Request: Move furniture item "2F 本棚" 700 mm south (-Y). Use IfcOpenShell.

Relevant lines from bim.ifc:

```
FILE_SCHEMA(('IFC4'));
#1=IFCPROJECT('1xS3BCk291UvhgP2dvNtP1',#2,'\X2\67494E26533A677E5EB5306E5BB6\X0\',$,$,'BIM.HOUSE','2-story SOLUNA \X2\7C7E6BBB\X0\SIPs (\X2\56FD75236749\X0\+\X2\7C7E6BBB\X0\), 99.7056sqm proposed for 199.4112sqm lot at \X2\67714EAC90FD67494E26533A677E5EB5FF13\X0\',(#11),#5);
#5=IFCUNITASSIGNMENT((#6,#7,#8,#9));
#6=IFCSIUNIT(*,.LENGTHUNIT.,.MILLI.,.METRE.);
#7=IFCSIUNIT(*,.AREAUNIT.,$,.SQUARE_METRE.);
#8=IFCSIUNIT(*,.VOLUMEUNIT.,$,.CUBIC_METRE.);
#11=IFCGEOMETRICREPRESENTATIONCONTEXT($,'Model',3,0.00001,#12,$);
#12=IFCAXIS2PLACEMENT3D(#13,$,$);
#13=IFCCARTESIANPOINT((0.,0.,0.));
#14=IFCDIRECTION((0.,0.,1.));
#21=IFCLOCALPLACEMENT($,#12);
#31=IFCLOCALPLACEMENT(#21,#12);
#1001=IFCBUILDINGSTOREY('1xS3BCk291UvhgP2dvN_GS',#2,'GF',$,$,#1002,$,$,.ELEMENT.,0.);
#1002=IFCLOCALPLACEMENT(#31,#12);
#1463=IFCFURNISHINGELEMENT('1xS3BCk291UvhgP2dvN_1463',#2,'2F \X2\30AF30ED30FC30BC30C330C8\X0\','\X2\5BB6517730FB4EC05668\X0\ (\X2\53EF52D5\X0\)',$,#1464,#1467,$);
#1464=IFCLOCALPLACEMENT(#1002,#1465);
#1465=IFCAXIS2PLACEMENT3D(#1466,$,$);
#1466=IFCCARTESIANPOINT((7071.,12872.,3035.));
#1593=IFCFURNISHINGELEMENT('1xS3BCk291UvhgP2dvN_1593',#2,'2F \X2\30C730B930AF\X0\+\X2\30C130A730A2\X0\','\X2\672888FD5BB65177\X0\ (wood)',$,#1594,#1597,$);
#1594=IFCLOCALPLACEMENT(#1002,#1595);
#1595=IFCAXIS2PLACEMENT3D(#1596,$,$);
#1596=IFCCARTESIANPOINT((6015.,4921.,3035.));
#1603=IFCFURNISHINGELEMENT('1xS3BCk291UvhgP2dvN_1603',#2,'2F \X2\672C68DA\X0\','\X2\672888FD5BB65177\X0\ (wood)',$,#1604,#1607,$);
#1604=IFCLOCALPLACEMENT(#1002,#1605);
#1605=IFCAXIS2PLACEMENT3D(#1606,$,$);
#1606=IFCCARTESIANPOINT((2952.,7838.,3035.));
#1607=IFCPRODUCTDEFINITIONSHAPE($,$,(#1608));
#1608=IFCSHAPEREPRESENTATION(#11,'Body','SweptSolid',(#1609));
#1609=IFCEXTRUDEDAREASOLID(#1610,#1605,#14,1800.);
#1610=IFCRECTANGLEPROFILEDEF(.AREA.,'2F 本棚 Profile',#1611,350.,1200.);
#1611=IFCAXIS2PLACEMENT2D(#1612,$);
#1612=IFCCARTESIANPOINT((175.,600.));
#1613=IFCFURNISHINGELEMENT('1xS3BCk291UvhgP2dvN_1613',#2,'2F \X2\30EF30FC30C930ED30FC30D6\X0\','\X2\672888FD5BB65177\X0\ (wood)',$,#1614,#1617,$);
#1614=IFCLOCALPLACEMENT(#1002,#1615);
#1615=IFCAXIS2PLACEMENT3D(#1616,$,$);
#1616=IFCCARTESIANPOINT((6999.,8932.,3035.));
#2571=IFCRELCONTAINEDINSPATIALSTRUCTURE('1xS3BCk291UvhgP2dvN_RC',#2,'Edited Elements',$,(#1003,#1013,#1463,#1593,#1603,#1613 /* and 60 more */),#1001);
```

```python
import ifcopenshell
import ifcopenshell.api.geometry
import ifcopenshell.util.placement
import ifcopenshell.util.unit

model = ifcopenshell.open("bim.ifc")
unit_scale = ifcopenshell.util.unit.calculate_unit_scale(model)

item = model.by_guid("1xS3BCk291UvhgP2dvN_1603")
matrix = ifcopenshell.util.placement.get_local_placement(item.ObjectPlacement)
matrix[1, 3] -= 0.7 / unit_scale
ifcopenshell.api.geometry.edit_object_placement(model, product=item, matrix=matrix, is_si=False)

print(ifcopenshell.util.placement.get_local_placement(item.ObjectPlacement).round(3) + 0.0)

model.write("bim_edited.ifc")
```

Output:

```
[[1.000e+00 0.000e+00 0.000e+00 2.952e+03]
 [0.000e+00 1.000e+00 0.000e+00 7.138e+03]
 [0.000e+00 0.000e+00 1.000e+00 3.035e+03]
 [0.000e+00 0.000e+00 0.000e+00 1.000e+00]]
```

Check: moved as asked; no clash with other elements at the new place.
